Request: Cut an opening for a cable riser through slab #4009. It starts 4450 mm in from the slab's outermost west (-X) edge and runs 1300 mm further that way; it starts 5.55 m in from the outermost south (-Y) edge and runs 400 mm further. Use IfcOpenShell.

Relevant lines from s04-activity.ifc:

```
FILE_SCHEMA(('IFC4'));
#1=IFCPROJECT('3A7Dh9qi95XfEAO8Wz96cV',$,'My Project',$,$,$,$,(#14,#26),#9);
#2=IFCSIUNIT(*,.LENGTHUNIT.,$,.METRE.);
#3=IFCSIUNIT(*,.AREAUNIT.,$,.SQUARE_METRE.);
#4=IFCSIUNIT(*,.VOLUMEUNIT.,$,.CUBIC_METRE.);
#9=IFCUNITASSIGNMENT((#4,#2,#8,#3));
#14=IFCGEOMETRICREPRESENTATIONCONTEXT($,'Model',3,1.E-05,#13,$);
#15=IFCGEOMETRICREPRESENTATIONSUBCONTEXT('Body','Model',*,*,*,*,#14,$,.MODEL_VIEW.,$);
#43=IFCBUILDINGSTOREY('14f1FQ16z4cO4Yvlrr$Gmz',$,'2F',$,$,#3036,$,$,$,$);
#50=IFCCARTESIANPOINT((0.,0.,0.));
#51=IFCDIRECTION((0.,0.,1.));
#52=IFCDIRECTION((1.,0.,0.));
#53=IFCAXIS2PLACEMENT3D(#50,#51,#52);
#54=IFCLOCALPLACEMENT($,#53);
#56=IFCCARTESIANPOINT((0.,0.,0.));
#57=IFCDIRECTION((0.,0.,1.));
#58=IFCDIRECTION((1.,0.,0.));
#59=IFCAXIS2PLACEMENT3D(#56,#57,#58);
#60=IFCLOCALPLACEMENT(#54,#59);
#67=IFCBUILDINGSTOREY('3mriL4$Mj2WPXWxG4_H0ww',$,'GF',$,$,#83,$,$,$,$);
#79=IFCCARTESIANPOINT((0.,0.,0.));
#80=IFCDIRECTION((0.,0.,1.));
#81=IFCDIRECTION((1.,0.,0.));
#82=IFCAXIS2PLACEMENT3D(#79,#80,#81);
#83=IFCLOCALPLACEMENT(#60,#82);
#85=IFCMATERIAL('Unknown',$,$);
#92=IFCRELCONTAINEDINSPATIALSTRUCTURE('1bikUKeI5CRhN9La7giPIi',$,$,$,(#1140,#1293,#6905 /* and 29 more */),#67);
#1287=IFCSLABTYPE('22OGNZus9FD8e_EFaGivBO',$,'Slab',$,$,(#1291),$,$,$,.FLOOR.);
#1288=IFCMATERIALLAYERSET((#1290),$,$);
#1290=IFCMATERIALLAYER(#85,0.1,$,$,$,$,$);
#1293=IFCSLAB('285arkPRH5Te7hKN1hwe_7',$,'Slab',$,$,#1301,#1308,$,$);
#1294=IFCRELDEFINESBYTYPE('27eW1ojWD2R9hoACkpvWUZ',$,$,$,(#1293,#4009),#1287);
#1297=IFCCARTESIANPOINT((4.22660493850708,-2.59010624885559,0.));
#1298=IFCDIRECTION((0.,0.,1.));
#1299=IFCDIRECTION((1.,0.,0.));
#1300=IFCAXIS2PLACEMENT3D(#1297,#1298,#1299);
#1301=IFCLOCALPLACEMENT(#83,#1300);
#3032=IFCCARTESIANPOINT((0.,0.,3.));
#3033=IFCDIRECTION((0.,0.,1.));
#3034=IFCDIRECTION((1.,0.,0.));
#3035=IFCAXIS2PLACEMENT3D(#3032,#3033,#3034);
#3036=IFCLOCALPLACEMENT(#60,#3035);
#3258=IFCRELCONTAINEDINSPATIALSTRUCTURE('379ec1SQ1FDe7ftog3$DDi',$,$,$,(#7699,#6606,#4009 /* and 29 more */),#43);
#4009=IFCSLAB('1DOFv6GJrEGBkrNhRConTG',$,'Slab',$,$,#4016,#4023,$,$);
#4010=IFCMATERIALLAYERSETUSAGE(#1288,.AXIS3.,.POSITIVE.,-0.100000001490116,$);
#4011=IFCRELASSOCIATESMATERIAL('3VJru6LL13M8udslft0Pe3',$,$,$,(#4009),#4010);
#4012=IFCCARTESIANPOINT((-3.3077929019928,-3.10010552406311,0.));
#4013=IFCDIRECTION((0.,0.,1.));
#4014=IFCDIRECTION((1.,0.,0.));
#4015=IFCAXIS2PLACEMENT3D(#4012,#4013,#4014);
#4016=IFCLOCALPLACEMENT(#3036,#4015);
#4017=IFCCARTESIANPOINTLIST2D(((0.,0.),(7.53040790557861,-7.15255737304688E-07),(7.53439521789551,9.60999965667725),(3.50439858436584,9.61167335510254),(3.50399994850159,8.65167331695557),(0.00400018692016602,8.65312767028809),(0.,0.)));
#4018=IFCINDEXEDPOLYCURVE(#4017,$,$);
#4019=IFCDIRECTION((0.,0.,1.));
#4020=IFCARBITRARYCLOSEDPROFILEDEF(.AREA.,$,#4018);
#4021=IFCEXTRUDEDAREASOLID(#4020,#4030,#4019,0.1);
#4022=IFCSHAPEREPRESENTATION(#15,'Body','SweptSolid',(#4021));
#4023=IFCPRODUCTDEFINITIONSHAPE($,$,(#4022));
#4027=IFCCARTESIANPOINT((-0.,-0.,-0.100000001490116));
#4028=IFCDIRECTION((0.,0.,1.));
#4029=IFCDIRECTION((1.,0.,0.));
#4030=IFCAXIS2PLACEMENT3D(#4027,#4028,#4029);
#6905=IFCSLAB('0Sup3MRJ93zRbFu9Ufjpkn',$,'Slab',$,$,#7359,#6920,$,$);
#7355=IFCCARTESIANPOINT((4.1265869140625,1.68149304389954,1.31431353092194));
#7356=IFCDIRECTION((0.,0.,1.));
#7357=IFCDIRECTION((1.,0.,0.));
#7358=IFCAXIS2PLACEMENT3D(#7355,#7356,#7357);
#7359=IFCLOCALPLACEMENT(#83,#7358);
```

```python
import numpy as np
import ifcopenshell
import ifcopenshell.api.feature
import ifcopenshell.api.geometry
import ifcopenshell.api.root
import ifcopenshell.geom
import ifcopenshell.util.placement
import ifcopenshell.util.representation
import ifcopenshell.util.shape
import ifcopenshell.util.unit

model = ifcopenshell.open("s04-activity.ifc")
unit_scale = ifcopenshell.util.unit.calculate_unit_scale(model)
settings = ifcopenshell.geom.settings()


def volume(element):
    """Net volume in cubic metres, openings subtracted."""
    shape = ifcopenshell.geom.create_shape(settings, element)
    return ifcopenshell.util.shape.get_volume(shape.geometry)


slab = model.by_id(4009)
before = volume(slab)

# Extent in the slab's own axes, in metres. The edges named are its -X and -Y sides.
slab_shape = ifcopenshell.geom.create_shape(settings, slab)
vertices = ifcopenshell.util.shape.get_vertices(slab_shape.geometry)
x_min, y_min, bottom = vertices.min(axis=0)
top = vertices[:, 2].max()

opening = ifcopenshell.api.root.create_entity(model, ifc_class="IfcOpeningElement", name="Cable riser opening", predefined_type="OPENING")
context = ifcopenshell.util.representation.get_context(model, "Model", "Body", "MODEL_VIEW")
width, depth = 1.3, 0.4
outline = [(0.0, 0.0), (width, 0.0), (width, depth), (0.0, depth), (0.0, 0.0)]
# Overshoot both faces by 50 mm so the cut is clean.
shape = ifcopenshell.api.geometry.add_slab_representation(
    model, context=context, depth=top - bottom + 0.1, polyline=outline
)
ifcopenshell.api.geometry.assign_representation(model, product=opening, representation=shape)

matrix = ifcopenshell.util.placement.get_local_placement(slab.ObjectPlacement)
matrix[:, 3] = matrix @ np.append(np.array([x_min + 4.45, y_min + 5.55, bottom - 0.05]) / unit_scale, 1.0)
ifcopenshell.api.geometry.edit_object_placement(model, product=opening, matrix=matrix, is_si=False)
ifcopenshell.api.feature.add_feature(model, feature=opening, element=slab)

after = volume(slab)

print(f"slab volume {before:.3f} -> {after:.3f} m3")

model.write("s04-activity_v2.ifc")
```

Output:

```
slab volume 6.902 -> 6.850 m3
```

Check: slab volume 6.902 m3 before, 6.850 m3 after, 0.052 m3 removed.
